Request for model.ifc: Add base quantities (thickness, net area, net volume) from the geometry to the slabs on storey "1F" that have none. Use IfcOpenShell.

First a look at what the model holds.

```python
import ifcopenshell
import ifcopenshell.util.element
import ifcopenshell.util.unit

model = ifcopenshell.open("model.ifc")
print(model.schema)
for unit_type in ("LENGTHUNIT", "AREAUNIT", "VOLUMEUNIT"):
    print(unit_type, ifcopenshell.util.unit.calculate_unit_scale(model, unit_type))
storey = next(s for s in model.by_type("IfcBuildingStorey") if s.Name == "1F")
slabs = [e for e in ifcopenshell.util.element.get_decomposition(storey) if e.is_a("IfcSlab")]
for e in sorted(slabs, key=lambda e: e.id()):
    print(e.id(), e.is_a(), e.Name, list(ifcopenshell.util.element.get_psets(e, qtos_only=True)), sep=" | ")
```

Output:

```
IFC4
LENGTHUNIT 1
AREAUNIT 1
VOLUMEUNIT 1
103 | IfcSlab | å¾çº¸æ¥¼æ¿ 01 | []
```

```python
import ifcopenshell
import ifcopenshell.api.pset
import ifcopenshell.geom
import ifcopenshell.util.element
import ifcopenshell.util.shape
import ifcopenshell.util.unit

model = ifcopenshell.open("model.ifc")
unit_scale = ifcopenshell.util.unit.calculate_unit_scale(model)
area_scale = ifcopenshell.util.unit.calculate_unit_scale(model, "AREAUNIT")
volume_scale = ifcopenshell.util.unit.calculate_unit_scale(model, "VOLUMEUNIT")
settings = ifcopenshell.geom.settings()

storey = next(s for s in model.by_type("IfcBuildingStorey") if s.Name == "1F")
slabs = [e for e in ifcopenshell.util.element.get_decomposition(storey) if e.is_a("IfcSlab")]

for e in sorted(slabs, key=lambda e: e.id()):
    if ifcopenshell.util.element.get_psets(e, qtos_only=True, should_inherit=False):
        continue
    # Geometry comes back in metres, in the element's own axes.
    shape = ifcopenshell.geom.create_shape(settings, e)
    values = {
        "Width": ifcopenshell.util.shape.get_z(shape.geometry) / unit_scale,
        "NetArea": ifcopenshell.util.shape.get_footprint_area(shape.geometry) / area_scale,
        "NetVolume": ifcopenshell.util.shape.get_volume(shape.geometry) / volume_scale,
    }
    qto = ifcopenshell.api.pset.add_qto(model, product=e, name="Qto_SlabBaseQuantities")
    ifcopenshell.api.pset.edit_qto(model, qto=qto, properties=values)
    print(e.id(), {k: round(v, 3) for k, v in values.items()})

model.write("model_updated.ifc")
```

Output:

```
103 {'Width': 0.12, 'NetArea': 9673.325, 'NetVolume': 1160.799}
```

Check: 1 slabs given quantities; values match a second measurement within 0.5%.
